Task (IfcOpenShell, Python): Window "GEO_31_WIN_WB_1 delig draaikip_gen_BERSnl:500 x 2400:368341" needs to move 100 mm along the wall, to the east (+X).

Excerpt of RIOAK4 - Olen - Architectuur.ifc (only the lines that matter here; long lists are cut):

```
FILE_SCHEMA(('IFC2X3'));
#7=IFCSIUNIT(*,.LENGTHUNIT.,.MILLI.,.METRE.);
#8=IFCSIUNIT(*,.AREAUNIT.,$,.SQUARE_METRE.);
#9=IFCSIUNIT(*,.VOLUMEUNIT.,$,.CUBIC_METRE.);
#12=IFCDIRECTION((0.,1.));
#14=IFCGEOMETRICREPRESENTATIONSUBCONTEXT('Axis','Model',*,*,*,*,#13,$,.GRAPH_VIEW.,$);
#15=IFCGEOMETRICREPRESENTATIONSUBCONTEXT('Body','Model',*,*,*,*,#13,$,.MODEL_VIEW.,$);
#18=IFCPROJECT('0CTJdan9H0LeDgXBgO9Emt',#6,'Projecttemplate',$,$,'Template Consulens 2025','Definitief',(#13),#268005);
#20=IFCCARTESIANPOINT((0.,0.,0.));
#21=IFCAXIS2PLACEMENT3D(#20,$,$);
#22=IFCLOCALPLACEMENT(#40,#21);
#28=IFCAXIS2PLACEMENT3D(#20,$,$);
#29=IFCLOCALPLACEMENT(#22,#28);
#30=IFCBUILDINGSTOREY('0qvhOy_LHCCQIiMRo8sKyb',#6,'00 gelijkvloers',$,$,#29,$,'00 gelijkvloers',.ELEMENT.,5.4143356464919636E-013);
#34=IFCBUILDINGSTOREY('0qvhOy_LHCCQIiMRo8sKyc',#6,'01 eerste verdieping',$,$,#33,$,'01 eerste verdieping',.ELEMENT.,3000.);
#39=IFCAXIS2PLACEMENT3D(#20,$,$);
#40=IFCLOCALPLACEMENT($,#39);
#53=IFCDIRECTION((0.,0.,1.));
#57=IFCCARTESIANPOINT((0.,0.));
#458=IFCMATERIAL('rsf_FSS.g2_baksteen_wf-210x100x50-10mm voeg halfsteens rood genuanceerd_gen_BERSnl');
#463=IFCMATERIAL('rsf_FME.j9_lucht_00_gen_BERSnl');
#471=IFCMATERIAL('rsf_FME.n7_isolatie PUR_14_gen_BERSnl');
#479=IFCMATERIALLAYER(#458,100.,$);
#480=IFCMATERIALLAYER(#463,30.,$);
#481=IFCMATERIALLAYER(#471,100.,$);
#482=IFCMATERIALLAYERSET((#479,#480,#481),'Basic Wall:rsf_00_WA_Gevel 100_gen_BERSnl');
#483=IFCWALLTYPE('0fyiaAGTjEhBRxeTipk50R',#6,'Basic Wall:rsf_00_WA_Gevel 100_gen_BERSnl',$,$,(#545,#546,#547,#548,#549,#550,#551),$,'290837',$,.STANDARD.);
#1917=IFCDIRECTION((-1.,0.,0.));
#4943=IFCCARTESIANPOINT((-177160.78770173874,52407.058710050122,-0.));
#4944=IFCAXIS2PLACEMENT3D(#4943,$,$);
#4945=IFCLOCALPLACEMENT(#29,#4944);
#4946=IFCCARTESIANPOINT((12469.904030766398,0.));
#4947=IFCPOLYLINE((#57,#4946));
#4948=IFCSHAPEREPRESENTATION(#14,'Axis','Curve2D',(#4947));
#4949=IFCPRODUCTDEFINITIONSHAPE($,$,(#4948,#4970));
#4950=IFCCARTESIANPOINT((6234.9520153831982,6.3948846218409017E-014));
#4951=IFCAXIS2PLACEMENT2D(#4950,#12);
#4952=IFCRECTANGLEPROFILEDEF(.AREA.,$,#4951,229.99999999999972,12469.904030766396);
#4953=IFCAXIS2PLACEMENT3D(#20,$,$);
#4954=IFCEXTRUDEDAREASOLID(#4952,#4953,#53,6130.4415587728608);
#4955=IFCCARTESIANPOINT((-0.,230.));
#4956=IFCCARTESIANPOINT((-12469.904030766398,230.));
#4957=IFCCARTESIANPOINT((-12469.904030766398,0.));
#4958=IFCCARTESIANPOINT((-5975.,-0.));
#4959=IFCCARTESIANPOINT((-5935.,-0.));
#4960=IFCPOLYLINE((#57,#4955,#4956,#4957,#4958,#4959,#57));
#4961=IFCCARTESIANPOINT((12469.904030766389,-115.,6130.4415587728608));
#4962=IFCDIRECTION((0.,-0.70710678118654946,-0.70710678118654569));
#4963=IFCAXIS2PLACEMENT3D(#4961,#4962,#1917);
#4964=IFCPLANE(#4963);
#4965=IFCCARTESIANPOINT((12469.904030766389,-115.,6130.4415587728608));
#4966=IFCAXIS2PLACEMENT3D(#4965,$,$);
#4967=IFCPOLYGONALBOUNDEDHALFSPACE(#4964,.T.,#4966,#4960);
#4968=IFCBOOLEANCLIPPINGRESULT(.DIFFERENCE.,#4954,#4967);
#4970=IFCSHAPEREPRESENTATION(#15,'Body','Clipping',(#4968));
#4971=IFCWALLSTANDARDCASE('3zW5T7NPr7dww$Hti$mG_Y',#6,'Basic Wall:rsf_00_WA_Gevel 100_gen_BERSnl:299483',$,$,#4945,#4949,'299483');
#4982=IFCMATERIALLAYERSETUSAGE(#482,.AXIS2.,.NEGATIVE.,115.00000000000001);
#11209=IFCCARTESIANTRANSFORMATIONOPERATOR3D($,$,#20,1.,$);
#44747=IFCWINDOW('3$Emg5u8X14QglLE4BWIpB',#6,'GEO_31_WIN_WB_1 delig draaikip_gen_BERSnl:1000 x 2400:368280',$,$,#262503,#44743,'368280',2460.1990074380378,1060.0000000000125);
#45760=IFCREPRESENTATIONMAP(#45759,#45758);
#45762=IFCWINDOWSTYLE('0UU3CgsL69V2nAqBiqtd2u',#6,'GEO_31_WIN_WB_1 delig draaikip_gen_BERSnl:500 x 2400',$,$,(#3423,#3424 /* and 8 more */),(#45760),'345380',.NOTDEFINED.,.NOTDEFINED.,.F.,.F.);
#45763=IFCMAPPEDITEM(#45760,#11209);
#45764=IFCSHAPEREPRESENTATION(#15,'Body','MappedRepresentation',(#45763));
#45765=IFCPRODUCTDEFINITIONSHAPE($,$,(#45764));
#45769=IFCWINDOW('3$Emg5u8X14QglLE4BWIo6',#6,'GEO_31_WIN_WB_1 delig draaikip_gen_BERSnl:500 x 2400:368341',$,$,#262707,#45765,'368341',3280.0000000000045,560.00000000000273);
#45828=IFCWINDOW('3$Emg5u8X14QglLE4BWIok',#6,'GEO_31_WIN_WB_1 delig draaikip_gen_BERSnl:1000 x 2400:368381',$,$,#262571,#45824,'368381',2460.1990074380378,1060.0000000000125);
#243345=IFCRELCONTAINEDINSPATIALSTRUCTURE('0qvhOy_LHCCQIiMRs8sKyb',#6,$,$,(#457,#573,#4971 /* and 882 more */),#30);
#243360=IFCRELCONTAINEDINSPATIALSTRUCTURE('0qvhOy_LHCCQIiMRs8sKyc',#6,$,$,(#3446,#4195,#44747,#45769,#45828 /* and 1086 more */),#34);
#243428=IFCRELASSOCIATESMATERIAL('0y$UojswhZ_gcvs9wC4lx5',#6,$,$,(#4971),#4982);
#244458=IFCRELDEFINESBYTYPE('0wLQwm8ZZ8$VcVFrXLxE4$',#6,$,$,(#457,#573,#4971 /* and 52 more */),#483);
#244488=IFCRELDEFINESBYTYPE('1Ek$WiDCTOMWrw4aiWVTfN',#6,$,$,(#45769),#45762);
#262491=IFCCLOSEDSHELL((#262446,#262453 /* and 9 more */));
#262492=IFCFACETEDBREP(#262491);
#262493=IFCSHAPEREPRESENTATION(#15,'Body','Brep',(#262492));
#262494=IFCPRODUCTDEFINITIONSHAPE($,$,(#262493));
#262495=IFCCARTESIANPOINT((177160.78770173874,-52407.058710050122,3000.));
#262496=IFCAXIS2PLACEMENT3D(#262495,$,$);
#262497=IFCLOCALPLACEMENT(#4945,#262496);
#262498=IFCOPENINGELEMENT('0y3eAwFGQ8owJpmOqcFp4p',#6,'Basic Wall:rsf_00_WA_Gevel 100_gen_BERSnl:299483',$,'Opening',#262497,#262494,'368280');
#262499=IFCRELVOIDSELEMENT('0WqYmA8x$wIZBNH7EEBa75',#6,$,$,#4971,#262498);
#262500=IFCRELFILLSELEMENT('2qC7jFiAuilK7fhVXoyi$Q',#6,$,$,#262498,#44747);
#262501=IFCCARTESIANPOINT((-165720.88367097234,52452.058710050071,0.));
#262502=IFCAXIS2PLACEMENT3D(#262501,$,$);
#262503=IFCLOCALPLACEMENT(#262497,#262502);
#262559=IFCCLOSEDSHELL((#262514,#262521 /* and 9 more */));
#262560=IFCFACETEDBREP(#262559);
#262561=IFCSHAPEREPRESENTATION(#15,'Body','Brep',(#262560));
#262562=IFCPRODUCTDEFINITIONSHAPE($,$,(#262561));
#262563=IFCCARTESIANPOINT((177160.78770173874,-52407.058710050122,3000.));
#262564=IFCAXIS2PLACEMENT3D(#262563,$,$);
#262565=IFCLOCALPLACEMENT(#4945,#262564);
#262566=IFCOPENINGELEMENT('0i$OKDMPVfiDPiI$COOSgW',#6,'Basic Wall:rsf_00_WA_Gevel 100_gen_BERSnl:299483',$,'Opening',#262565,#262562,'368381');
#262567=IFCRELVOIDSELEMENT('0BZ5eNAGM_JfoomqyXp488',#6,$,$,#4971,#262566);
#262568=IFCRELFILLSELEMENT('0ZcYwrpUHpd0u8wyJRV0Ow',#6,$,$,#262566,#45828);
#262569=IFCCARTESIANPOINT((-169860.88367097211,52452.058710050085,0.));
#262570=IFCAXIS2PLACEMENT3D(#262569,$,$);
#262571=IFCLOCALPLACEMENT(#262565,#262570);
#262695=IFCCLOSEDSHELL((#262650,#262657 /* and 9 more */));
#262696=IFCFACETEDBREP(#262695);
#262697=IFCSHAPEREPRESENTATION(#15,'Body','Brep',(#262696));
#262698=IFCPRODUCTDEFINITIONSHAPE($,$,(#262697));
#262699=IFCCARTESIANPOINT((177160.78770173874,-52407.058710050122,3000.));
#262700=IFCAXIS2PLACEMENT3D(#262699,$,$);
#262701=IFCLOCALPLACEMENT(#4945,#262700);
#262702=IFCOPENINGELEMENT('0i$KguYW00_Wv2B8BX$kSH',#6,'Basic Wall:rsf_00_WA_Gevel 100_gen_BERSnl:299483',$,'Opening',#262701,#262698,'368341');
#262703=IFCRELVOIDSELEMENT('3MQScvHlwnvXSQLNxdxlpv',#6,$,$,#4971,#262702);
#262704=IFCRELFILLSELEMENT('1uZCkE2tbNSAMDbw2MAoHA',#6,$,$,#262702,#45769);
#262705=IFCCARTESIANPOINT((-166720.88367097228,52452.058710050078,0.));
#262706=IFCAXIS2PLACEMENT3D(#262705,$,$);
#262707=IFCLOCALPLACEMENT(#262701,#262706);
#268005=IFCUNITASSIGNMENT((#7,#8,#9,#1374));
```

```python
import ifcopenshell
import ifcopenshell.api.geometry
import ifcopenshell.util.placement

model = ifcopenshell.open("RIOAK4 - Olen - Architectuur.ifc")

window = model.by_guid("3$Emg5u8X14QglLE4BWIo6")
opening = window.FillsVoids[0].RelatingOpeningElement
wall = opening.VoidsElements[0].RelatingBuildingElement

wall_matrix = ifcopenshell.util.placement.get_local_placement(wall.ObjectPlacement)
shift = wall_matrix[:3, 0] * 100.0
before = ifcopenshell.util.placement.get_local_placement(window.ObjectPlacement)[:3, 3].copy()

# The window is placed relative to its opening, so it follows when the opening moves.
matrix = ifcopenshell.util.placement.get_local_placement(opening.ObjectPlacement)
matrix[:3, 3] += shift
ifcopenshell.api.geometry.edit_object_placement(
    model, product=opening, matrix=matrix, is_si=False, should_transform_children=True
)

after = ifcopenshell.util.placement.get_local_placement(window.ObjectPlacement)[:3, 3]
print("window moved by", (after - before).round(3) + 0.0)

model.write("RIOAK4 - Olen - Architectuur_v2.ifc")
```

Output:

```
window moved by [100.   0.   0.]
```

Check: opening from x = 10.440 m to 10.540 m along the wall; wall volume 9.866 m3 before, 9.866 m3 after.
